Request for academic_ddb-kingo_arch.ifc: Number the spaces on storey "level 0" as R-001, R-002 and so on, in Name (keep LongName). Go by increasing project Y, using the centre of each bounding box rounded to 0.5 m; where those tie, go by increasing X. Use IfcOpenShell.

First a look at what the model holds.

```python
import ifcopenshell
import ifcopenshell.util.element
import ifcopenshell.util.placement

model = ifcopenshell.open("academic_ddb-kingo_arch.ifc")
print(model.schema)
storey = next(s for s in model.by_type("IfcBuildingStorey") if s.Name == "level 0")
spaces = [e for e in ifcopenshell.util.element.get_decomposition(storey) if e.is_a("IfcSpace")]
for e in sorted(spaces, key=lambda e: e.id()):
    origin = ifcopenshell.util.placement.get_local_placement(e.ObjectPlacement)[:3, 3]
    print(e.id(), e.Name, e.LongName, origin.round(2) + 0.0, sep=" | ")
```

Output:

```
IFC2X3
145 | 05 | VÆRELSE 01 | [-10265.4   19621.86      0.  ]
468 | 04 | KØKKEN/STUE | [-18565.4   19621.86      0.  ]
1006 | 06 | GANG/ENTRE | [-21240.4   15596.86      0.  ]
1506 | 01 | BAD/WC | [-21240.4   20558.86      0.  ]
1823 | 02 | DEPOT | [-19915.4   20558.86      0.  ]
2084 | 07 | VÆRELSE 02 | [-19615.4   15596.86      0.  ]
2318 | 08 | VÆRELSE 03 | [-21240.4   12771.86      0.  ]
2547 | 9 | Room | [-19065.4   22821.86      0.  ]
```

```python
import ifcopenshell
import ifcopenshell.geom
import ifcopenshell.util.element
import ifcopenshell.util.shape

model = ifcopenshell.open("academic_ddb-kingo_arch.ifc")
settings = ifcopenshell.geom.settings()
settings.set("use-world-coords", True)


def centre(element):
    shape = ifcopenshell.geom.create_shape(settings, element)
    return ifcopenshell.util.shape.get_bbox_centroid(shape.geometry)


storey = next(s for s in model.by_type("IfcBuildingStorey") if s.Name == "level 0")
spaces = [e for e in ifcopenshell.util.element.get_decomposition(storey) if e.is_a("IfcSpace")]

# Insertion points can sit at a corner or the storey origin, so sort by the geometry (in metres).
centres = {e: centre(e) for e in spaces}
spaces.sort(key=lambda e: (round(centres[e][1] / 0.5), centres[e][0]))

for i, e in enumerate(spaces, start=1):
    number = f"R-0{i:02d}"
    e.Name = number
    print(e.id(), number)

model.write("academic_ddb-kingo_arch_edited.ifc")
```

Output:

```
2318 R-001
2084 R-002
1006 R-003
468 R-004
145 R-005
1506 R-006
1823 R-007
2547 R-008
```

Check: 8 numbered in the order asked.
